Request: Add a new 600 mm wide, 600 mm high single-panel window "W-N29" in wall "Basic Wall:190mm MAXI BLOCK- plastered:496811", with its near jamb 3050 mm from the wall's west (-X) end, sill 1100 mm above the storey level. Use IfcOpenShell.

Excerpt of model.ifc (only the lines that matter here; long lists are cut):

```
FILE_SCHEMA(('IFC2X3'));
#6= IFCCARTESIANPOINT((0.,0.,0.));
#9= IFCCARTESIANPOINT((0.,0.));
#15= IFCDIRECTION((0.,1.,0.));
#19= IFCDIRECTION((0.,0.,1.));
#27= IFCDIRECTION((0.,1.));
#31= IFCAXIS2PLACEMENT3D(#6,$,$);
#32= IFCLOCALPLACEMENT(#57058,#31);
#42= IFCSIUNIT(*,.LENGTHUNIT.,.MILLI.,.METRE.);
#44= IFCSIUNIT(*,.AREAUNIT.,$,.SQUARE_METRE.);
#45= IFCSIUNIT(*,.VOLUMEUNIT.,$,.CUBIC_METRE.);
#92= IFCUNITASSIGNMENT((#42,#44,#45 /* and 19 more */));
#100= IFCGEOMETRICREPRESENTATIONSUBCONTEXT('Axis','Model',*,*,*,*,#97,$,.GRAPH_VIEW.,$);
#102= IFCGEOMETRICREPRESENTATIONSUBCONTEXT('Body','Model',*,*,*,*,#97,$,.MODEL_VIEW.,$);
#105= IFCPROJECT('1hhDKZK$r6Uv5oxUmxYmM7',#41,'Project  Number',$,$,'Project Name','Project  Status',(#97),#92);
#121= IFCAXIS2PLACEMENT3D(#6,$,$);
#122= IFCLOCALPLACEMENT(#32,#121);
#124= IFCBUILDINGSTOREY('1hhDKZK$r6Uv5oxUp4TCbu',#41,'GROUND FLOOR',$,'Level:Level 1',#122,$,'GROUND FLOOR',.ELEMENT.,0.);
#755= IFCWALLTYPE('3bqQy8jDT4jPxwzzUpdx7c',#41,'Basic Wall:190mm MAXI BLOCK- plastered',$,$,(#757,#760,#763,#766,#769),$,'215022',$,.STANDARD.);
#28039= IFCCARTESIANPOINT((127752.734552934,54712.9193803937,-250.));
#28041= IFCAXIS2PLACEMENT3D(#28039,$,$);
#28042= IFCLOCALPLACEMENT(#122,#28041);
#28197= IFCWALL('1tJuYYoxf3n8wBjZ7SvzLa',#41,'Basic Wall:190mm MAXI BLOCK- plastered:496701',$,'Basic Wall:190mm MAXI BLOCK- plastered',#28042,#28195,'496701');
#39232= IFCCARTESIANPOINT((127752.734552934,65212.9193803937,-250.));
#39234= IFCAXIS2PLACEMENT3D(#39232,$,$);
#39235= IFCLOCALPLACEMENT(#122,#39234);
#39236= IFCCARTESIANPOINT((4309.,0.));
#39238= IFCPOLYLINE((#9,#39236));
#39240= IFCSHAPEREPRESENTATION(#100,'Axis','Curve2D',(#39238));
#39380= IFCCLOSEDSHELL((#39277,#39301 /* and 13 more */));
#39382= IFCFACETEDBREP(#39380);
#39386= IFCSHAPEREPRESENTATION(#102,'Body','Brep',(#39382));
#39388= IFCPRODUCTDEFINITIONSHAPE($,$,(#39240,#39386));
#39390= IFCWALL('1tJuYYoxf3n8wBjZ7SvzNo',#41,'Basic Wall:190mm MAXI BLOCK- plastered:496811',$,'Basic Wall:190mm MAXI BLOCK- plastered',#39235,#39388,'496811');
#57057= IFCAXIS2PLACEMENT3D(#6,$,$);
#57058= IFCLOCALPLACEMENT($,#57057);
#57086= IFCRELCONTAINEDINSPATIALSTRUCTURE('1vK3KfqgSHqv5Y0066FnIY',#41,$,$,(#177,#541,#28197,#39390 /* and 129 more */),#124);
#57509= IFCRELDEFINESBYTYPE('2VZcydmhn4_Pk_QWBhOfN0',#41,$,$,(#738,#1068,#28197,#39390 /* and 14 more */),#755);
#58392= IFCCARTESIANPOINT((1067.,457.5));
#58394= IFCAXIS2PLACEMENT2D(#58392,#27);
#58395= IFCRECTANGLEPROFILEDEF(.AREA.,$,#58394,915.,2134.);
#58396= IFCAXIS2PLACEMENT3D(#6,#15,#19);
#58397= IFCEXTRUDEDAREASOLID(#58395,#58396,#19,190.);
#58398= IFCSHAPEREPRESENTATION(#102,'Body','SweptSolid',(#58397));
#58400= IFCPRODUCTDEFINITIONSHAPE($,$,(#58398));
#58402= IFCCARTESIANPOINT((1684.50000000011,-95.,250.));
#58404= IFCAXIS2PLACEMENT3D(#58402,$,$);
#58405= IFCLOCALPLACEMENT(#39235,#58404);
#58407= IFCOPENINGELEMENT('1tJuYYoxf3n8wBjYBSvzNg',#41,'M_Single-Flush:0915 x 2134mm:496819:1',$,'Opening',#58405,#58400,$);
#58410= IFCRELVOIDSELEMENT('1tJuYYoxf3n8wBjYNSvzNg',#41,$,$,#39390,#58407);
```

```python
import numpy as np
import ifcopenshell
import ifcopenshell.api.feature
import ifcopenshell.api.geometry
import ifcopenshell.api.root
import ifcopenshell.api.spatial
import ifcopenshell.api.type
import ifcopenshell.geom
import ifcopenshell.util.element
import ifcopenshell.util.placement
import ifcopenshell.util.representation
import ifcopenshell.util.shape
import ifcopenshell.util.unit

model = ifcopenshell.open("model.ifc")
unit_scale = ifcopenshell.util.unit.calculate_unit_scale(model)
settings = ifcopenshell.geom.settings()


def volume(element):
    """Net volume in cubic metres, openings subtracted."""
    shape = ifcopenshell.geom.create_shape(settings, element)
    return ifcopenshell.util.shape.get_volume(shape.geometry)


wall = model.by_id(39390)
storey = ifcopenshell.util.element.get_container(wall, ifc_class="IfcBuildingStorey")
context = ifcopenshell.util.representation.get_context(model, "Model", "Body", "MODEL_VIEW")
before = volume(wall)

width, height, from_end, sill = 0.6, 0.6, 3.05, 1.1  # metres

# The wall runs along its own X axis, and the end named is its -X end.
wall_shape = ifcopenshell.geom.create_shape(settings, wall)
x, y, z = ifcopenshell.util.shape.get_vertices(wall_shape.geometry).T
start = x.min() + from_end
face, thickness = float(y.min()), float(y.max() - y.min())
wall_matrix = ifcopenshell.util.placement.get_local_placement(wall.ObjectPlacement)
level = ifcopenshell.util.placement.get_local_placement(storey.ObjectPlacement)[2, 3]


def in_wall(x, y):
    """Placement at x, y metres in the wall's axes, at sill height."""
    matrix = wall_matrix.copy()
    matrix[:, 3] = wall_matrix @ np.array([x / unit_scale, y / unit_scale, 0.0, 1.0])
    matrix[2, 3] = level + sill / unit_scale
    return matrix


# Opening: a box that overshoots both wall faces by 50 mm.
opening = ifcopenshell.api.root.create_entity(model, ifc_class="IfcOpeningElement")
box = ifcopenshell.api.geometry.add_wall_representation(
    model, context=context, length=width, height=height, thickness=thickness + 0.1
)
ifcopenshell.api.geometry.assign_representation(model, product=opening, representation=box)
ifcopenshell.api.geometry.edit_object_placement(model, product=opening, matrix=in_wall(start, face - 0.05), is_si=False)
ifcopenshell.api.feature.add_feature(model, feature=opening, element=wall)

window = ifcopenshell.api.root.create_entity(model, ifc_class="IfcWindow", name="W-N29")
window.OverallWidth, window.OverallHeight = width / unit_scale, height / unit_scale
body = ifcopenshell.api.geometry.add_window_representation(
    model,
    context=context,
    overall_width=window.OverallWidth,
    overall_height=window.OverallHeight,
    partition_type="SINGLE_PANEL",
)
ifcopenshell.api.geometry.assign_representation(model, product=window, representation=body)
ifcopenshell.api.spatial.assign_container(model, products=[window], relating_structure=storey)
fills = ifcopenshell.api.feature.add_filling(model, opening=opening, element=window)
fills.OwnerHistory = window.OwnerHistory  # required in IFC2X3

# IFC2X3 keeps the operation on the window style.
style = ifcopenshell.api.root.create_entity(model, ifc_class="IfcWindowStyle", name="W-N29")
style.OperationType, style.ConstructionType = "SINGLE_PANEL", "NOTDEFINED"
style.ParameterTakesPrecedence = style.Sizeable = False
ifcopenshell.api.type.assign_type(model, related_objects=[window], relating_type=style)

# Centre the window in the wall's thickness.
ifcopenshell.api.geometry.edit_object_placement(model, product=window, matrix=in_wall(start, face), is_si=False)
window_shape = ifcopenshell.geom.create_shape(settings, window)
depth = ifcopenshell.util.shape.get_vertices(window_shape.geometry)[:, 1]
offset = face + thickness / 2 - (depth.min() + depth.max()) / 2
ifcopenshell.api.geometry.edit_object_placement(model, product=window, matrix=in_wall(start, offset), is_si=False)

after = volume(wall)

print(f"wall volume {before:.3f} -> {after:.3f} m3")

model.write("model_updated.ifc")
```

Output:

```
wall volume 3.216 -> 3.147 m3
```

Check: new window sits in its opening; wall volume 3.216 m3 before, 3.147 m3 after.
